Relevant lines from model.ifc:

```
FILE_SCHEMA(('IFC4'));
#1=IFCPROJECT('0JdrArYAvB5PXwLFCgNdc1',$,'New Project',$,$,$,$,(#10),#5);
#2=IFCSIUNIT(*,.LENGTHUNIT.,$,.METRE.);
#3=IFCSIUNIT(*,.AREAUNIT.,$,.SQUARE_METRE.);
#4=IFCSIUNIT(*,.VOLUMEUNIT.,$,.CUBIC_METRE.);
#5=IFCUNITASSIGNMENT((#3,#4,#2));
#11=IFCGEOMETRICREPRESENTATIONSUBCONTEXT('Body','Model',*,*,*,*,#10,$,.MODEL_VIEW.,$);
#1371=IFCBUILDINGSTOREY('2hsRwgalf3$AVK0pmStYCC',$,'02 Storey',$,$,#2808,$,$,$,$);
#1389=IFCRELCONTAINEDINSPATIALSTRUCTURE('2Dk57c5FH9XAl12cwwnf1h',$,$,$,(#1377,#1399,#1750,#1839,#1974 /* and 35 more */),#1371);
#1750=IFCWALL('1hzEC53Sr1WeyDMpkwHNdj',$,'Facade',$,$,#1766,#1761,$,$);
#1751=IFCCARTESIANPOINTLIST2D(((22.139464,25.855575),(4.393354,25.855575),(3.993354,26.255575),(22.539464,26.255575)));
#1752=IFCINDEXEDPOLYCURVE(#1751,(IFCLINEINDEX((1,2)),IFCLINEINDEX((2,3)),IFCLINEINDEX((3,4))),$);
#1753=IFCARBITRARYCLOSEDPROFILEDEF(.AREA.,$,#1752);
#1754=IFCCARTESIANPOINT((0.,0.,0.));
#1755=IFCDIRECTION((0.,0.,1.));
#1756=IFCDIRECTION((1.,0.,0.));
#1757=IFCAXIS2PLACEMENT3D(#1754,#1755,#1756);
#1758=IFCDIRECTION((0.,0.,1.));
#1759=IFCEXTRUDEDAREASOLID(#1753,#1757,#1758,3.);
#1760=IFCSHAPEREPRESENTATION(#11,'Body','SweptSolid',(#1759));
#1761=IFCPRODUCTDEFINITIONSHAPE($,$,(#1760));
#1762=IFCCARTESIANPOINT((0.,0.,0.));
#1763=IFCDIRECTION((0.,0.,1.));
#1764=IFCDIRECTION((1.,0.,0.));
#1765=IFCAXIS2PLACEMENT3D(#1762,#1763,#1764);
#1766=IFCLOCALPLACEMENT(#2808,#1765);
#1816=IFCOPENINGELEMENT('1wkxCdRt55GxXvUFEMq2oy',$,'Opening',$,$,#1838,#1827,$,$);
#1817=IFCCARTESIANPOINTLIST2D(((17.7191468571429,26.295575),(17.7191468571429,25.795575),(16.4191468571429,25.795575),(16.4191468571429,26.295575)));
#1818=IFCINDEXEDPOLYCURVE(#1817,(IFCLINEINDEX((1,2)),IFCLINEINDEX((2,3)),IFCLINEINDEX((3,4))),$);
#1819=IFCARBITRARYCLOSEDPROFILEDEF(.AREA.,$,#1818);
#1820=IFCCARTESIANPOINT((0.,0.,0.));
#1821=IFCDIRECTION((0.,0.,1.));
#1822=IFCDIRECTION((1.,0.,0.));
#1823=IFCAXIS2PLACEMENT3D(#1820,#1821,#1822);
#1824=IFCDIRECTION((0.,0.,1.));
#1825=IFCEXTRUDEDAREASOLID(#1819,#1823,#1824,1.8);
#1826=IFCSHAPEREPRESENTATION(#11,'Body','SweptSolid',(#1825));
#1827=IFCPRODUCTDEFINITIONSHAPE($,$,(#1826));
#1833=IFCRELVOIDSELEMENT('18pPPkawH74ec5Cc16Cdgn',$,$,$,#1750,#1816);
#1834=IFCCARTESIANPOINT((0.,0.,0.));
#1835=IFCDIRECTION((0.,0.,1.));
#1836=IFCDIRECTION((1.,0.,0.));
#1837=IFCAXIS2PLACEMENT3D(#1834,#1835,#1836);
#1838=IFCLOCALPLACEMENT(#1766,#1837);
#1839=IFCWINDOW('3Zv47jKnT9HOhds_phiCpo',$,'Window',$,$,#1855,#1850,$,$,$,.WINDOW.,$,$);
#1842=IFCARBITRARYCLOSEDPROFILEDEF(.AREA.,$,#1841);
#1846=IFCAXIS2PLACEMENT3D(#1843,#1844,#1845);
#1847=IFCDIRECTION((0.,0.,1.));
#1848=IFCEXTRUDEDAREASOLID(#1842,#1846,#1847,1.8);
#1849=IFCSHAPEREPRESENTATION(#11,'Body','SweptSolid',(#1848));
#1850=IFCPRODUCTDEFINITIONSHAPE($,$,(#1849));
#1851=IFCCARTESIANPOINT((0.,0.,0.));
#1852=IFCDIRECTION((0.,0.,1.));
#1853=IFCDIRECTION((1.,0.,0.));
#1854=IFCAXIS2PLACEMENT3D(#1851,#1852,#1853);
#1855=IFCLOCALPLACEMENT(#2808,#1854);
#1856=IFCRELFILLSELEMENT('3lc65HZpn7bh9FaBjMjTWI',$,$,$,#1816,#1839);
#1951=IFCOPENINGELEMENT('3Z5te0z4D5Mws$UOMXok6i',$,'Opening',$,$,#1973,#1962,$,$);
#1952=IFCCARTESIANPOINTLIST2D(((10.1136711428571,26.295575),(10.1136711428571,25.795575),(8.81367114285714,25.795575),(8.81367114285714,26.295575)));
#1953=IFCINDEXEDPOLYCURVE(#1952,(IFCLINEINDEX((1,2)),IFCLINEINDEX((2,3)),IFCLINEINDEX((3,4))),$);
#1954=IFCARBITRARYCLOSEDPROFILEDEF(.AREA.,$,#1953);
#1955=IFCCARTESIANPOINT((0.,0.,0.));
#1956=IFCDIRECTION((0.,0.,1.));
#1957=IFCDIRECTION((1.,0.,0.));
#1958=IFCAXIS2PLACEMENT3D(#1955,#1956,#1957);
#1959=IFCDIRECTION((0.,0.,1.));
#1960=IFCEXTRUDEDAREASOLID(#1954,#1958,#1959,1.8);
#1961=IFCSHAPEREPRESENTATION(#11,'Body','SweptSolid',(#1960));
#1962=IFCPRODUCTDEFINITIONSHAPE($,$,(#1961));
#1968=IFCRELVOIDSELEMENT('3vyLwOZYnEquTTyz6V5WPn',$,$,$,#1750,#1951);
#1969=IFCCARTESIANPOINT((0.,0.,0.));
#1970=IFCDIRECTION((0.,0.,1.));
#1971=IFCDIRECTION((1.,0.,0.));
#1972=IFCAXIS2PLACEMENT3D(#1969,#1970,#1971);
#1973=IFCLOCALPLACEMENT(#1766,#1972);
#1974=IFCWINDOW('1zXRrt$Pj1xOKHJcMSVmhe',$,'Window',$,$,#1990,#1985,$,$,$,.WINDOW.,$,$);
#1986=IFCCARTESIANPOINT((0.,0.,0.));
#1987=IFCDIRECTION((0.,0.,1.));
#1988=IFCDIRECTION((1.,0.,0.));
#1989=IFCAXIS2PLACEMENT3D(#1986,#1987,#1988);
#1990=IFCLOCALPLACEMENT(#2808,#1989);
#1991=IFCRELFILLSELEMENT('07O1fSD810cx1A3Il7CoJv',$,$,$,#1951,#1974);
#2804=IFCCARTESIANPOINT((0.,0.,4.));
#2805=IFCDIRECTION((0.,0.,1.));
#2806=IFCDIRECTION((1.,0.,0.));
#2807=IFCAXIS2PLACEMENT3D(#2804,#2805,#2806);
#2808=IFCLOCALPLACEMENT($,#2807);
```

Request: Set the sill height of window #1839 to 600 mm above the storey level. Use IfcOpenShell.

```python
import numpy as np
import ifcopenshell
import ifcopenshell.api.geometry
import ifcopenshell.geom
import ifcopenshell.util.element
import ifcopenshell.util.placement
import ifcopenshell.util.shape
import ifcopenshell.util.unit

model = ifcopenshell.open("model.ifc")
unit_scale = ifcopenshell.util.unit.calculate_unit_scale(model)

window = model.by_id(1839)
opening = window.FillsVoids[0].RelatingOpeningElement
storey = ifcopenshell.util.element.get_container(window, ifc_class="IfcBuildingStorey")
level = ifcopenshell.util.placement.get_local_placement(storey.ObjectPlacement)[2, 3]

# The opening's origin need not be at the sill, so measure its lowest point.
shape = ifcopenshell.geom.create_shape(ifcopenshell.geom.settings(), opening)
bottom = ifcopenshell.util.shape.get_shape_bottom_elevation(shape, shape.geometry) / unit_scale
dz = level + 0.6 - bottom

shift = np.array([0.0, 0.0, dz])
# The window is not placed relative to its opening, so move both.
for product in (opening, window):
    matrix = ifcopenshell.util.placement.get_local_placement(product.ObjectPlacement)
    matrix[:3, 3] += shift
    ifcopenshell.api.geometry.edit_object_placement(model, product=product, matrix=matrix, is_si=False)

print(f"moved by {dz * unit_scale:+.3f} m")

model.write("model_edited.ifc")
```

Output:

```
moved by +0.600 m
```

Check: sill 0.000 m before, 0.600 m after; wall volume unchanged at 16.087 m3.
